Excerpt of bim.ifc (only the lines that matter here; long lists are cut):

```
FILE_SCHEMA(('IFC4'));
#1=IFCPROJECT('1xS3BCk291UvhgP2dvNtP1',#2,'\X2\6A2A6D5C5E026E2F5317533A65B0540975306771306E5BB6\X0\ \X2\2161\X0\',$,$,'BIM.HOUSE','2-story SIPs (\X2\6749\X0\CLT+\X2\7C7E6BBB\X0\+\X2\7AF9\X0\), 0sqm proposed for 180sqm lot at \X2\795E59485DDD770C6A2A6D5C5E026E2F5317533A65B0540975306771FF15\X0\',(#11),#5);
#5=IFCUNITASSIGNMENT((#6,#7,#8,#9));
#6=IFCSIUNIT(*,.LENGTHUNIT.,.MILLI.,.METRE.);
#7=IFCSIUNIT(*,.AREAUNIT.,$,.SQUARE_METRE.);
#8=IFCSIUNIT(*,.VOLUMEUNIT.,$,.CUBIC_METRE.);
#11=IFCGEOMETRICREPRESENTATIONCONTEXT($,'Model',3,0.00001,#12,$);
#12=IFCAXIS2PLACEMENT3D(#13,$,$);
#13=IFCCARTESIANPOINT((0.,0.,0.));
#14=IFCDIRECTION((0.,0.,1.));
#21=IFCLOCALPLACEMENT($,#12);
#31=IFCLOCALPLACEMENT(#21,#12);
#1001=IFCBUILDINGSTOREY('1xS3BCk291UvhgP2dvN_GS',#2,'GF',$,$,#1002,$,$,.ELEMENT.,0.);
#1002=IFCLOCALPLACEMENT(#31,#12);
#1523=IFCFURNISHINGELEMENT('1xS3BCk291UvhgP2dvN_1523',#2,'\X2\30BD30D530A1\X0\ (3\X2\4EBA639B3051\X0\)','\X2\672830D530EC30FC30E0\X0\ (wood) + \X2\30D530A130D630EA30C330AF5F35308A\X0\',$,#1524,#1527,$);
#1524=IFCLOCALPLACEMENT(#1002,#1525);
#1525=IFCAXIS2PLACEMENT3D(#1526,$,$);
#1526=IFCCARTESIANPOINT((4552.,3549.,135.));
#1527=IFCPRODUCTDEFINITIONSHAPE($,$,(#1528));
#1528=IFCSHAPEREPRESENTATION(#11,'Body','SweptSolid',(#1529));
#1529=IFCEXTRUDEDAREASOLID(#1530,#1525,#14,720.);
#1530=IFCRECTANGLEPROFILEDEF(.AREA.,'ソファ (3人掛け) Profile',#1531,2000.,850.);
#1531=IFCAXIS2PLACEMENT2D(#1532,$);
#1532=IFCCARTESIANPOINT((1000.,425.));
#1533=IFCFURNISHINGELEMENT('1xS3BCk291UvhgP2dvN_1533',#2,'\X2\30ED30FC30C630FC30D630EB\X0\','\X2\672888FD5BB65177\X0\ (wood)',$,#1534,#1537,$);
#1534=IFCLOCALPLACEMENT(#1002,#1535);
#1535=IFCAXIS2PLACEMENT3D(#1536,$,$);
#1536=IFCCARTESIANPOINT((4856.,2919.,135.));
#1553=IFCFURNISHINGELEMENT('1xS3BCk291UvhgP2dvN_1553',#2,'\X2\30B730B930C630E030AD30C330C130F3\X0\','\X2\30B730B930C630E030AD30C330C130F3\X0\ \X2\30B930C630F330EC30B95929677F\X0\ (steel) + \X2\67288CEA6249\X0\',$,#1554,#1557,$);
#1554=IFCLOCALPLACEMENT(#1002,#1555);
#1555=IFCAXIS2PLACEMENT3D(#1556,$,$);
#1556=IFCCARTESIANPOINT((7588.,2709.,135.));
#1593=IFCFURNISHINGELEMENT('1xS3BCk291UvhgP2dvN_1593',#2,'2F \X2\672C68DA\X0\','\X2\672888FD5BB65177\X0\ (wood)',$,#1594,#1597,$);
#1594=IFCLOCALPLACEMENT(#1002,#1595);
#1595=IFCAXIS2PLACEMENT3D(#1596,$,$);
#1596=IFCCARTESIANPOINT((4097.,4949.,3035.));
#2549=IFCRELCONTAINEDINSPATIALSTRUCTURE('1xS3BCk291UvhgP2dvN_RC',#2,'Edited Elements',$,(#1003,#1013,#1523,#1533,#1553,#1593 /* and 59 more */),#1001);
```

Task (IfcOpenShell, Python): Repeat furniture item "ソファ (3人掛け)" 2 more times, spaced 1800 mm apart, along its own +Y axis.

```python
import ifcopenshell
import ifcopenshell.api.geometry
import ifcopenshell.api.root
import ifcopenshell.util.element
import ifcopenshell.util.placement

model = ifcopenshell.open("bim.ifc")


def reuse_history(source, copy):
    """copy_class also copies each property set's owner history, people and application; keep the originals."""
    for rel in copy.IsDefinedBy:
        if rel.is_a("IfcRelDefinesByProperties") and (history := rel.RelatingPropertyDefinition.OwnerHistory):
            rel.RelatingPropertyDefinition.OwnerHistory = source.OwnerHistory
            ifcopenshell.util.element.remove_deep2(model, history)


source = model.by_id(1523)
base = ifcopenshell.util.placement.get_local_placement(source.ObjectPlacement)
step = base[:3, 1] * 1800.0

for i in range(1, 3):
    copy = ifcopenshell.api.root.copy_class(model, product=source)
    copy.Representation = ifcopenshell.util.element.copy_deep(
        model, source.Representation, exclude=["IfcGeometricRepresentationContext", "IfcRepresentationMap"]
    )
    reuse_history(source, copy)
    matrix = base.copy()
    matrix[:3, 3] += i * step
    print("added at", matrix[:3, 3].round(3) + 0.0)
    ifcopenshell.api.geometry.edit_object_placement(model, product=copy, matrix=matrix, is_si=False)

model.write("bim_edited.ifc")
```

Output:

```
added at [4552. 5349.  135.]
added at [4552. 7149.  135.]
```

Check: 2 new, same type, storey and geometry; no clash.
